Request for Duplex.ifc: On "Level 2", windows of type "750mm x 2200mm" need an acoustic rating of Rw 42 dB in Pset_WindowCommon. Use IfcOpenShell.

First a look at what the model holds.

```python
import ifcopenshell
import ifcopenshell.util.element

model = ifcopenshell.open("Duplex.ifc")
print(model.schema)
storey = next(s for s in model.by_type("IfcBuildingStorey") if s.Name == "Level 2")
windows = [e for e in ifcopenshell.util.element.get_decomposition(storey) if e.is_a("IfcWindow")]
seen = {}
for e in windows:
    element_type = ifcopenshell.util.element.get_type(e)
    key = (element_type.Name if element_type != e and element_type else None, ifcopenshell.util.element.get_pset(e, "Pset_WindowCommon", "AcousticRating"))
    seen[key] = seen.get(key, 0) + 1
for (name, value), count in sorted(seen.items(), key=str):
    print(count, "x", name, "|", value)
```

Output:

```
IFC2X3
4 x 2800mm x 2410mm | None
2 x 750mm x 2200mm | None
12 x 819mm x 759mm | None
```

```python
import ifcopenshell
import ifcopenshell.api.pset
import ifcopenshell.util.element

model = ifcopenshell.open("Duplex.ifc")

storey = next(s for s in model.by_type("IfcBuildingStorey") if s.Name == "Level 2")
windows = [e for e in ifcopenshell.util.element.get_decomposition(storey) if e.is_a("IfcWindow")]

count = 0
for e in windows:
    element_type = ifcopenshell.util.element.get_type(e)
    if element_type in (None, e) or element_type.Name != "750mm x 2200mm":
        continue
    # add_pset returns the element's existing set when there is one.
    pset = ifcopenshell.api.pset.add_pset(model, product=e, name="Pset_WindowCommon")
    ifcopenshell.api.pset.edit_pset(model, pset=pset, properties={"AcousticRating": "Rw 42 dB"})
    count += 1

print(count, "windows updated")

model.write("Duplex_updated.ifc")
```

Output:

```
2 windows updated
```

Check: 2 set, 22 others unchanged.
